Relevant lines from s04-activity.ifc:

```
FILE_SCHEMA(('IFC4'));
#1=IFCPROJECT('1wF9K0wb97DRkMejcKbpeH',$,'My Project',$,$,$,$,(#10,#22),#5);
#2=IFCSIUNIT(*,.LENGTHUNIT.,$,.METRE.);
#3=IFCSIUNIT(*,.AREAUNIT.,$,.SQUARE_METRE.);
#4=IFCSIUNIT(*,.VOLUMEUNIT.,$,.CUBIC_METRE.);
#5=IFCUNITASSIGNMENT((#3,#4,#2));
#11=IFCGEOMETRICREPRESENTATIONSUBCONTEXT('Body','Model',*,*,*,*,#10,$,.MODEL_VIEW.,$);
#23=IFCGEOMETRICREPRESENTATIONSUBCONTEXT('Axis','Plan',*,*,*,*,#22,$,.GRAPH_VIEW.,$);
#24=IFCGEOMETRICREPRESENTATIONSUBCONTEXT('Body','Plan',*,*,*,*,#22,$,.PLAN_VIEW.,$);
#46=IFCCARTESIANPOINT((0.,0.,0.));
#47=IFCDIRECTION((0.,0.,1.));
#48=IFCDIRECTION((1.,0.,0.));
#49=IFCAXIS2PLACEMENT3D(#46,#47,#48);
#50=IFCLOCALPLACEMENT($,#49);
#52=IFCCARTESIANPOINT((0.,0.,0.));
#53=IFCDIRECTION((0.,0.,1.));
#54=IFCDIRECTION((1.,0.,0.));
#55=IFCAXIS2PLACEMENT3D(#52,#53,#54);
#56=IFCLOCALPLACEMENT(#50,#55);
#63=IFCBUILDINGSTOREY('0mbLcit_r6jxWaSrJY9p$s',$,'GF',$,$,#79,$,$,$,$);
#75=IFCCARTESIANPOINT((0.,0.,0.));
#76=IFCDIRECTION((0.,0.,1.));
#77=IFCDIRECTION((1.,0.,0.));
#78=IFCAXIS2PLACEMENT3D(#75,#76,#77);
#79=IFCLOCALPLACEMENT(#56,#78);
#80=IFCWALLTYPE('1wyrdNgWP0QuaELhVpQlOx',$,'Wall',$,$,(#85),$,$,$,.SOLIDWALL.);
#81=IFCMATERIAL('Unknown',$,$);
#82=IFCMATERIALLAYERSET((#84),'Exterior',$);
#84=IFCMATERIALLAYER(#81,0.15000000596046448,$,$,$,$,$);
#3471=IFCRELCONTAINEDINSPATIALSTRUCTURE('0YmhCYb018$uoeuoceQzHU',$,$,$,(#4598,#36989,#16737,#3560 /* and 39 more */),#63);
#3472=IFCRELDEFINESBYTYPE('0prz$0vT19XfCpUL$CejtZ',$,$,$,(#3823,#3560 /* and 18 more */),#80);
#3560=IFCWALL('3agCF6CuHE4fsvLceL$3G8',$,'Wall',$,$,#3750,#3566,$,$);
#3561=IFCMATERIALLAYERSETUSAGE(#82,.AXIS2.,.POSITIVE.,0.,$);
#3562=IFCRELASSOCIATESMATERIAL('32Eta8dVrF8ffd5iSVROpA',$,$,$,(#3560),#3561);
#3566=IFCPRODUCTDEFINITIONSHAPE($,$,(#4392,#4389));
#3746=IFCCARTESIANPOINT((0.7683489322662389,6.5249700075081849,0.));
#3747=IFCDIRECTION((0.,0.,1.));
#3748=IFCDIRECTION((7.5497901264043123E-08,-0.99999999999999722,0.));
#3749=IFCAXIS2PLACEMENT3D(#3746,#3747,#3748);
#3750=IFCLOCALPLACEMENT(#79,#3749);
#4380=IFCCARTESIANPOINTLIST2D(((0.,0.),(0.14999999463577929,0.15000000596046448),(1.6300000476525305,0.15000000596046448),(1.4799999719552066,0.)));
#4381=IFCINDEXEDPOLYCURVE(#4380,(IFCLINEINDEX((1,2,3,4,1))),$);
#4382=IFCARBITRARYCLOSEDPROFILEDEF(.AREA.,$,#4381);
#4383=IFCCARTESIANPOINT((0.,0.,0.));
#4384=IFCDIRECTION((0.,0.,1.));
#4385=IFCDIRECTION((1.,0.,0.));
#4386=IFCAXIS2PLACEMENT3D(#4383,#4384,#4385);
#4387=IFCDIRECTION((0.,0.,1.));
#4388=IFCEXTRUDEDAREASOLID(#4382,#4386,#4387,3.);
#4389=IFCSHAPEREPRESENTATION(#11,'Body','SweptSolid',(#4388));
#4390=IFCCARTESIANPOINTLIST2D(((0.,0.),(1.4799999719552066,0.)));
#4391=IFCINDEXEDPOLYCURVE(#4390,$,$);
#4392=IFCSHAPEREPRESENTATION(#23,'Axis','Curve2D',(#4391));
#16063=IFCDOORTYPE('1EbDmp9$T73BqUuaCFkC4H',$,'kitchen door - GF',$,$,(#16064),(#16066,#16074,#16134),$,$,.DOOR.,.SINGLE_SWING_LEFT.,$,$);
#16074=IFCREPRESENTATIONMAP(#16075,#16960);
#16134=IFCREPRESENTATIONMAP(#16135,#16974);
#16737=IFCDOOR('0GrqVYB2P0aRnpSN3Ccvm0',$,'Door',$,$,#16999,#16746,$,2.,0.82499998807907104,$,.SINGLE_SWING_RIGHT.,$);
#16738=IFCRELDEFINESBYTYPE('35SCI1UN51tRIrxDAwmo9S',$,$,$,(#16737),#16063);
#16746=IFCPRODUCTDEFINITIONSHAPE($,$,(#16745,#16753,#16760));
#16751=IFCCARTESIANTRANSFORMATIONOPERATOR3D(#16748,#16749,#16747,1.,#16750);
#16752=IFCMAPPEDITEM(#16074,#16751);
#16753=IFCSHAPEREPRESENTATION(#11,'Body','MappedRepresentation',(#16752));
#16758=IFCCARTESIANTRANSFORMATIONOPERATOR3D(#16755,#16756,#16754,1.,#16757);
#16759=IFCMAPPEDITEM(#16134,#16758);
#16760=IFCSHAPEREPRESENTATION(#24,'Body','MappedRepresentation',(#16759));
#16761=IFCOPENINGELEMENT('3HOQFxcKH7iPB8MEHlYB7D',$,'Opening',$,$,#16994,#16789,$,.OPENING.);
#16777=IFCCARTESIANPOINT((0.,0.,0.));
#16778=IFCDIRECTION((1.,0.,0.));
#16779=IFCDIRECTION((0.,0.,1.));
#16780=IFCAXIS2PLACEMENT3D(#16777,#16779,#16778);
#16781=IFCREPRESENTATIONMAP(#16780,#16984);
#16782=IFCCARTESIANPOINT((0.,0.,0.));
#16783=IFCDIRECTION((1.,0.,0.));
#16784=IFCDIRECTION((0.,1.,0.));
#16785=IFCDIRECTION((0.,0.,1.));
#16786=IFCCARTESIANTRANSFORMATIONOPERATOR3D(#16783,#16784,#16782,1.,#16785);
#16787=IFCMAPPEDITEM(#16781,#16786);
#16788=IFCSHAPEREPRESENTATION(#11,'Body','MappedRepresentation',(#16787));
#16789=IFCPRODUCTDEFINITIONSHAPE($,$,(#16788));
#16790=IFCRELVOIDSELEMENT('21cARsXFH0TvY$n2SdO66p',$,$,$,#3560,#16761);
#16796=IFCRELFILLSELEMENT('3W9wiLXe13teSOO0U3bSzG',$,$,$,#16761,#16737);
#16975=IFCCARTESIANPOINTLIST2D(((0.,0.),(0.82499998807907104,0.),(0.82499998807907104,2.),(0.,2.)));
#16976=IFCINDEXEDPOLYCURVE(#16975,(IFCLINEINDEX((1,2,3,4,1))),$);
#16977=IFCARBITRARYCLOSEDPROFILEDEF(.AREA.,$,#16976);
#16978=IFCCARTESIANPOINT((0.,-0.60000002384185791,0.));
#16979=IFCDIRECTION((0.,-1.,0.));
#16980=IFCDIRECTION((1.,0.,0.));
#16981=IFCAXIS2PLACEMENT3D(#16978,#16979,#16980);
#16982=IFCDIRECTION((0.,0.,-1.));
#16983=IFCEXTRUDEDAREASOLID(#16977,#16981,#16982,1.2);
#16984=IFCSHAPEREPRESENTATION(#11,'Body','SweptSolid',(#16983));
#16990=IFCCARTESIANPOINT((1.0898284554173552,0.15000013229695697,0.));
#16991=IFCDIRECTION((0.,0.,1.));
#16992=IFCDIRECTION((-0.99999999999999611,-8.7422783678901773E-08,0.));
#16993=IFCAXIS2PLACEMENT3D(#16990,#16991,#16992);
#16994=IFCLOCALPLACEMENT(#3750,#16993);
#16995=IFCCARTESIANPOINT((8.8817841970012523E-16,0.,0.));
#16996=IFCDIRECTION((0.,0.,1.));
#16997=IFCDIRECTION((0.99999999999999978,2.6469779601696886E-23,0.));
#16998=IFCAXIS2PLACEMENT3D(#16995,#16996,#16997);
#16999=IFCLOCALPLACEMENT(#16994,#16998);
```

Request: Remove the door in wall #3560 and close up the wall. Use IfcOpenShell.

```python
import ifcopenshell
import ifcopenshell.api.feature
import ifcopenshell.api.root
import ifcopenshell.geom
import ifcopenshell.util.shape

model = ifcopenshell.open("s04-activity.ifc")
settings = ifcopenshell.geom.settings()


def volume(element):
    """Net volume in cubic metres, openings subtracted."""
    shape = ifcopenshell.geom.create_shape(settings, element)
    return ifcopenshell.util.shape.get_volume(shape.geometry)


door = model.by_guid("0GrqVYB2P0aRnpSN3Ccvm0")
opening = door.FillsVoids[0].RelatingOpeningElement
wall = opening.VoidsElements[0].RelatingBuildingElement
before = volume(wall)

ifcopenshell.api.root.remove_product(model, product=door)
ifcopenshell.api.feature.remove_feature(model, feature=opening)

after = volume(wall)

print(f"wall volume {before:.3f} -> {after:.3f} m3")

model.write("s04-activity-out.ifc")
```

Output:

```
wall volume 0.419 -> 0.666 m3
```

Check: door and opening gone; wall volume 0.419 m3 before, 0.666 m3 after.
